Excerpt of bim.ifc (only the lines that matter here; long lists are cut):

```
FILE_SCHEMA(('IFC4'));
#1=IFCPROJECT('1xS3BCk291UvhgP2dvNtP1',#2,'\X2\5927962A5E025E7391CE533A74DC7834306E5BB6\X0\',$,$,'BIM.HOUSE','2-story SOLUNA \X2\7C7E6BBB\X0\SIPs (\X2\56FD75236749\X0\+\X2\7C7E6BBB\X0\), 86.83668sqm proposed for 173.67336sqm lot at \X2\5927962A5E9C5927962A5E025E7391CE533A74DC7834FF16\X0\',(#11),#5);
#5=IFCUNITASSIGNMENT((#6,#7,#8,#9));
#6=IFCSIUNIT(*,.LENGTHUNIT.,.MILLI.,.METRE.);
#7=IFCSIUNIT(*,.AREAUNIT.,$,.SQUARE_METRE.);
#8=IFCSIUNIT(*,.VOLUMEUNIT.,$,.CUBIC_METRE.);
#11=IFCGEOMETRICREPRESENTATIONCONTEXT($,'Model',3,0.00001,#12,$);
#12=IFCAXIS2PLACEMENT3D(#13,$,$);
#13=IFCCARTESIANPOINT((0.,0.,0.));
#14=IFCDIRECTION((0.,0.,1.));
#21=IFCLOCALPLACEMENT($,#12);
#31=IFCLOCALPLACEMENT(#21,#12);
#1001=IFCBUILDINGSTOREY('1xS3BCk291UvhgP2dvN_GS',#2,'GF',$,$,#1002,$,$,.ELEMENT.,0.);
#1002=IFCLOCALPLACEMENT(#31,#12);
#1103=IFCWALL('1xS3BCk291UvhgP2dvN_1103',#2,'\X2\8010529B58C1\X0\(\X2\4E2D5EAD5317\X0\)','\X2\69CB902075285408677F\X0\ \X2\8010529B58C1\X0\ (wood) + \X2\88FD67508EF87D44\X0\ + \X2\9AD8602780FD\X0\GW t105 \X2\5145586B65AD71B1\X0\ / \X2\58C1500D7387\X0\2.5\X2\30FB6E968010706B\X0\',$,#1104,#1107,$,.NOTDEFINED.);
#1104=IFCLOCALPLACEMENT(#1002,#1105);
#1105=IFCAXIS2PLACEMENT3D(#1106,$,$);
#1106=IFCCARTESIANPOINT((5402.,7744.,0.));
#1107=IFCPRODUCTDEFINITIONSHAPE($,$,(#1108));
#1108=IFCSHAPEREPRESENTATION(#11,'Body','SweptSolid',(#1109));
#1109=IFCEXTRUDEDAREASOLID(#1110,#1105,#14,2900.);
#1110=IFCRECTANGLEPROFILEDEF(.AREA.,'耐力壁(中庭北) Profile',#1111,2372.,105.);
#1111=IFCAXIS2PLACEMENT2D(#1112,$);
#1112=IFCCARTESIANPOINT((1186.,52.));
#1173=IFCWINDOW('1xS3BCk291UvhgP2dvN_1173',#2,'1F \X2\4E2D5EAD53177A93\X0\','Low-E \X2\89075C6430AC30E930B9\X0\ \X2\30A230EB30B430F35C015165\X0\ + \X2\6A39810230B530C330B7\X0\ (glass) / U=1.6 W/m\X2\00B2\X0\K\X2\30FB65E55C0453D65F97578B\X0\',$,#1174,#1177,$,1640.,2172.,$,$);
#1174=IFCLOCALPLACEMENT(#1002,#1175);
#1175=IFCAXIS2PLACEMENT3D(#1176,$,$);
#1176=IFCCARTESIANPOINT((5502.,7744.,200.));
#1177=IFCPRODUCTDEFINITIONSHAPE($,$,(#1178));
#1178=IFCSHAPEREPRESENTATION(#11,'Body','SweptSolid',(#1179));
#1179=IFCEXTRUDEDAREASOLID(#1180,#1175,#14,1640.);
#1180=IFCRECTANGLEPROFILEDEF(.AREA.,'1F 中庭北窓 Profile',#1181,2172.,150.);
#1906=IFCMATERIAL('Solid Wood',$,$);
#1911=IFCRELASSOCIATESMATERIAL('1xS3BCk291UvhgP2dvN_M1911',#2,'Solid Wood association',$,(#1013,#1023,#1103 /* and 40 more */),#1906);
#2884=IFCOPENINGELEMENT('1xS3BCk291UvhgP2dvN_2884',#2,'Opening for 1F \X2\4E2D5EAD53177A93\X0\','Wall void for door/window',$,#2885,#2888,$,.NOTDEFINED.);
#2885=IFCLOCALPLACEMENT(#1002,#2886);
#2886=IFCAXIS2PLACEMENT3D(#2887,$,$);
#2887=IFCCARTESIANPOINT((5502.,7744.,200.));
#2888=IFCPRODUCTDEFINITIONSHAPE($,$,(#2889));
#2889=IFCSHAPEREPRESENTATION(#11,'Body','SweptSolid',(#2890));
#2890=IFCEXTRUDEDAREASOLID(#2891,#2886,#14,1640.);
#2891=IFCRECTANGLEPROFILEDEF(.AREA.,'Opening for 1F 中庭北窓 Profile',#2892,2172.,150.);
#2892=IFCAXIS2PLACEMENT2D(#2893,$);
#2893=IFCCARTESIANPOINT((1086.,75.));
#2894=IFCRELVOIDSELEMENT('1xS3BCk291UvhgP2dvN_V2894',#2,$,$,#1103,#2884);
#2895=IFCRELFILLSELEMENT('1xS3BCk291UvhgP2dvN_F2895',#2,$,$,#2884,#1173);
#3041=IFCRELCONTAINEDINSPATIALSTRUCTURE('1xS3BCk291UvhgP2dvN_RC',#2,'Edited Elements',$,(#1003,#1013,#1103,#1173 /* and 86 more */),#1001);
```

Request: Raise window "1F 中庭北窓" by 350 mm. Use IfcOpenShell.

```python
import numpy as np
import ifcopenshell
import ifcopenshell.api.geometry
import ifcopenshell.util.placement
import ifcopenshell.util.unit

model = ifcopenshell.open("bim.ifc")
unit_scale = ifcopenshell.util.unit.calculate_unit_scale(model)

window = model.by_guid("1xS3BCk291UvhgP2dvN_1173")
opening = window.FillsVoids[0].RelatingOpeningElement
dz = 350.0

shift = np.array([0.0, 0.0, dz])
# The window is not placed relative to its opening, so move both.
for product in (opening, window):
    matrix = ifcopenshell.util.placement.get_local_placement(product.ObjectPlacement)
    matrix[:3, 3] += shift
    ifcopenshell.api.geometry.edit_object_placement(model, product=product, matrix=matrix, is_si=False)

print(f"moved by {dz * unit_scale:+.3f} m")

model.write("bim-out.ifc")
```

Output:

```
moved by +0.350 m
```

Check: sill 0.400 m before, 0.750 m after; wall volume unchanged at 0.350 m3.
